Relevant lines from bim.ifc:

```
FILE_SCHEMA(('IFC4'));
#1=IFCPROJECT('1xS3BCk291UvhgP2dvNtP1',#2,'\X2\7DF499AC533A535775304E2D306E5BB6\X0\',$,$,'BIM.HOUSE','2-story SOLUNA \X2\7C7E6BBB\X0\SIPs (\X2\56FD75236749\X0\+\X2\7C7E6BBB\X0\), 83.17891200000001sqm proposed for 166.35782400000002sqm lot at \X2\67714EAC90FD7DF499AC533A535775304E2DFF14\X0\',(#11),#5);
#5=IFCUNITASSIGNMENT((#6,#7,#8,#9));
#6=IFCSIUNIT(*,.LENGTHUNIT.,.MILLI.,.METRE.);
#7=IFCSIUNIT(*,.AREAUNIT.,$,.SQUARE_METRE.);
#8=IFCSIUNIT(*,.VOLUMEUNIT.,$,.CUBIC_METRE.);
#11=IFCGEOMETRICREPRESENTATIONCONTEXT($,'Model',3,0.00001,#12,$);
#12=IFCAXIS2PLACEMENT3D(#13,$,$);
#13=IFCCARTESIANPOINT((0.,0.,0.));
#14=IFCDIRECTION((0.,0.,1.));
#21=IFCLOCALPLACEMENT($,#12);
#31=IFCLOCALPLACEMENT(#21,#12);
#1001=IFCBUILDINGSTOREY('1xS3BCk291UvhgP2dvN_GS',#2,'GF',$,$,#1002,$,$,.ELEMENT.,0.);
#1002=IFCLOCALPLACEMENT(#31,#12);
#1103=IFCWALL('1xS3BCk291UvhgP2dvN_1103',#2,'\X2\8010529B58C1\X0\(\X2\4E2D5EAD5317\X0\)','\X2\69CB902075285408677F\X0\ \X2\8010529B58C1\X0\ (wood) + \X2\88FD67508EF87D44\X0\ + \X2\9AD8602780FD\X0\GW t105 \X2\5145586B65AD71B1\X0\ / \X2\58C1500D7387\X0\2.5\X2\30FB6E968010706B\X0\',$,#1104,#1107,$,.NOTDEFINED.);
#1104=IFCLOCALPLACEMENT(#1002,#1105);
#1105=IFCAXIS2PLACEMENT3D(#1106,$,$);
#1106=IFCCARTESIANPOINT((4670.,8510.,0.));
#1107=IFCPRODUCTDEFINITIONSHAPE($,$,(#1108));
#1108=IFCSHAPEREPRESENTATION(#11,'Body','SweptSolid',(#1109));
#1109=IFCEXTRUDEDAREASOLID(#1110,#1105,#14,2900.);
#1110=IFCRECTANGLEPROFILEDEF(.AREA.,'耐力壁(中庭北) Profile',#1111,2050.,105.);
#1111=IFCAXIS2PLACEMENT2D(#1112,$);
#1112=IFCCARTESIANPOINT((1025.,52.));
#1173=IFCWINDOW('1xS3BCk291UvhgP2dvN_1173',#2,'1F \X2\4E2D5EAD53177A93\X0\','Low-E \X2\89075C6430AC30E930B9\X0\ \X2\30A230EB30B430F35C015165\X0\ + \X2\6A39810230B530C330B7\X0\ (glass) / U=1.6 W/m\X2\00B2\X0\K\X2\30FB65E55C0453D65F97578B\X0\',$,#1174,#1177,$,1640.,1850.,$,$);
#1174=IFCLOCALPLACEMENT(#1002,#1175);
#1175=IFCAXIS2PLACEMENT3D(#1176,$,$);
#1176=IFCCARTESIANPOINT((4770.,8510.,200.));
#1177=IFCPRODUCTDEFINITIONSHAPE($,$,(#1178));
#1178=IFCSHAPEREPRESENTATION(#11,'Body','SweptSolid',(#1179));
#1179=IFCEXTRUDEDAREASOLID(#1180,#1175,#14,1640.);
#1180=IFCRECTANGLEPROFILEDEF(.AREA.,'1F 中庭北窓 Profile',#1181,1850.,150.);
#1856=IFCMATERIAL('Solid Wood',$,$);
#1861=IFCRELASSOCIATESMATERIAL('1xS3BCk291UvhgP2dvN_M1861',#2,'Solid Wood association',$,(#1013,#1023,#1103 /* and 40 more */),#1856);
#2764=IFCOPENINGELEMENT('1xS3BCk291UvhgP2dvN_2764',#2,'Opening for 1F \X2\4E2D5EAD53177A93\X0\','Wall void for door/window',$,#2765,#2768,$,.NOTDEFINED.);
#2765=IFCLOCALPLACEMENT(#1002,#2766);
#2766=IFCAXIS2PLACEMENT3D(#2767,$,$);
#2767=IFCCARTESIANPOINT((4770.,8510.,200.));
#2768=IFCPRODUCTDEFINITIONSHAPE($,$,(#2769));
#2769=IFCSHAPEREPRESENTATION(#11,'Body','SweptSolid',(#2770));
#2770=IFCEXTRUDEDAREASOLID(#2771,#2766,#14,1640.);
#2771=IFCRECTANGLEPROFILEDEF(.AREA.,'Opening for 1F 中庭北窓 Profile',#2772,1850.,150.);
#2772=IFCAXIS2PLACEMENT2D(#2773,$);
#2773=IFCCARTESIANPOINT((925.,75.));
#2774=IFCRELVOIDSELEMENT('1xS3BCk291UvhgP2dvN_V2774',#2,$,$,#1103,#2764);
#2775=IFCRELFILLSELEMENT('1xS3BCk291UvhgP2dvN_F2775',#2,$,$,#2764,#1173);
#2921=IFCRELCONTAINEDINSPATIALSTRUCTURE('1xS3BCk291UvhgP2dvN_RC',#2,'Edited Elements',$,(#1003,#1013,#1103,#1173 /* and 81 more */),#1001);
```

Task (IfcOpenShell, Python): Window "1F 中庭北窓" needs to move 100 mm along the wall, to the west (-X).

```python
import ifcopenshell
import ifcopenshell.api.geometry
import ifcopenshell.util.placement

model = ifcopenshell.open("bim.ifc")

window = model.by_guid("1xS3BCk291UvhgP2dvN_1173")
opening = window.FillsVoids[0].RelatingOpeningElement
wall = opening.VoidsElements[0].RelatingBuildingElement

wall_matrix = ifcopenshell.util.placement.get_local_placement(wall.ObjectPlacement)
shift = wall_matrix[:3, 0] * -100.0
before = ifcopenshell.util.placement.get_local_placement(window.ObjectPlacement)[:3, 3].copy()

# The window is not placed relative to its opening, so move both.
for product in (opening, window):
    matrix = ifcopenshell.util.placement.get_local_placement(product.ObjectPlacement)
    matrix[:3, 3] += shift
    ifcopenshell.api.geometry.edit_object_placement(model, product=product, matrix=matrix, is_si=False)

after = ifcopenshell.util.placement.get_local_placement(window.ObjectPlacement)[:3, 3]
print("window moved by", (after - before).round(3) + 0.0)

model.write("bim-out.ifc")
```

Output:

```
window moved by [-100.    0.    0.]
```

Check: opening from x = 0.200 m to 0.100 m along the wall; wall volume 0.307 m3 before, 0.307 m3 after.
